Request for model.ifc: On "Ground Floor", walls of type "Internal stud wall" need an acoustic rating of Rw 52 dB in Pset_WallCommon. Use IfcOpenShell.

First a look at what the model holds.

```python
import ifcopenshell
import ifcopenshell.util.element

model = ifcopenshell.open("model.ifc")
print(model.schema)
storey = next(s for s in model.by_type("IfcBuildingStorey") if s.Name == "Ground Floor")
walls = [e for e in ifcopenshell.util.element.get_decomposition(storey) if e.is_a("IfcWall")]
seen = {}
for e in walls:
    element_type = ifcopenshell.util.element.get_type(e)
    key = (element_type.Name if element_type != e and element_type else None, ifcopenshell.util.element.get_pset(e, "Pset_WallCommon", "AcousticRating"))
    seen[key] = seen.get(key, 0) + 1
for (name, value), count in sorted(seen.items(), key=str):
    print(count, "x", name, "|", value)
```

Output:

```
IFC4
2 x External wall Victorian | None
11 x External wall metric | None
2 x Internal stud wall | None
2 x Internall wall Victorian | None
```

```python
import ifcopenshell
import ifcopenshell.api.pset
import ifcopenshell.util.element

model = ifcopenshell.open("model.ifc")

storey = next(s for s in model.by_type("IfcBuildingStorey") if s.Name == "Ground Floor")
walls = [e for e in ifcopenshell.util.element.get_decomposition(storey) if e.is_a("IfcWall")]

count = 0
for e in walls:
    element_type = ifcopenshell.util.element.get_type(e)
    if element_type in (None, e) or element_type.Name != "Internal stud wall":
        continue
    # add_pset returns the element's existing set when there is one.
    pset = ifcopenshell.api.pset.add_pset(model, product=e, name="Pset_WallCommon")
    ifcopenshell.api.pset.edit_pset(model, pset=pset, properties={"AcousticRating": "Rw 52 dB"})
    count += 1

print(count, "walls updated")

model.write("model_edited.ifc")
```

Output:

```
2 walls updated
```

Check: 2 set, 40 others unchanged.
